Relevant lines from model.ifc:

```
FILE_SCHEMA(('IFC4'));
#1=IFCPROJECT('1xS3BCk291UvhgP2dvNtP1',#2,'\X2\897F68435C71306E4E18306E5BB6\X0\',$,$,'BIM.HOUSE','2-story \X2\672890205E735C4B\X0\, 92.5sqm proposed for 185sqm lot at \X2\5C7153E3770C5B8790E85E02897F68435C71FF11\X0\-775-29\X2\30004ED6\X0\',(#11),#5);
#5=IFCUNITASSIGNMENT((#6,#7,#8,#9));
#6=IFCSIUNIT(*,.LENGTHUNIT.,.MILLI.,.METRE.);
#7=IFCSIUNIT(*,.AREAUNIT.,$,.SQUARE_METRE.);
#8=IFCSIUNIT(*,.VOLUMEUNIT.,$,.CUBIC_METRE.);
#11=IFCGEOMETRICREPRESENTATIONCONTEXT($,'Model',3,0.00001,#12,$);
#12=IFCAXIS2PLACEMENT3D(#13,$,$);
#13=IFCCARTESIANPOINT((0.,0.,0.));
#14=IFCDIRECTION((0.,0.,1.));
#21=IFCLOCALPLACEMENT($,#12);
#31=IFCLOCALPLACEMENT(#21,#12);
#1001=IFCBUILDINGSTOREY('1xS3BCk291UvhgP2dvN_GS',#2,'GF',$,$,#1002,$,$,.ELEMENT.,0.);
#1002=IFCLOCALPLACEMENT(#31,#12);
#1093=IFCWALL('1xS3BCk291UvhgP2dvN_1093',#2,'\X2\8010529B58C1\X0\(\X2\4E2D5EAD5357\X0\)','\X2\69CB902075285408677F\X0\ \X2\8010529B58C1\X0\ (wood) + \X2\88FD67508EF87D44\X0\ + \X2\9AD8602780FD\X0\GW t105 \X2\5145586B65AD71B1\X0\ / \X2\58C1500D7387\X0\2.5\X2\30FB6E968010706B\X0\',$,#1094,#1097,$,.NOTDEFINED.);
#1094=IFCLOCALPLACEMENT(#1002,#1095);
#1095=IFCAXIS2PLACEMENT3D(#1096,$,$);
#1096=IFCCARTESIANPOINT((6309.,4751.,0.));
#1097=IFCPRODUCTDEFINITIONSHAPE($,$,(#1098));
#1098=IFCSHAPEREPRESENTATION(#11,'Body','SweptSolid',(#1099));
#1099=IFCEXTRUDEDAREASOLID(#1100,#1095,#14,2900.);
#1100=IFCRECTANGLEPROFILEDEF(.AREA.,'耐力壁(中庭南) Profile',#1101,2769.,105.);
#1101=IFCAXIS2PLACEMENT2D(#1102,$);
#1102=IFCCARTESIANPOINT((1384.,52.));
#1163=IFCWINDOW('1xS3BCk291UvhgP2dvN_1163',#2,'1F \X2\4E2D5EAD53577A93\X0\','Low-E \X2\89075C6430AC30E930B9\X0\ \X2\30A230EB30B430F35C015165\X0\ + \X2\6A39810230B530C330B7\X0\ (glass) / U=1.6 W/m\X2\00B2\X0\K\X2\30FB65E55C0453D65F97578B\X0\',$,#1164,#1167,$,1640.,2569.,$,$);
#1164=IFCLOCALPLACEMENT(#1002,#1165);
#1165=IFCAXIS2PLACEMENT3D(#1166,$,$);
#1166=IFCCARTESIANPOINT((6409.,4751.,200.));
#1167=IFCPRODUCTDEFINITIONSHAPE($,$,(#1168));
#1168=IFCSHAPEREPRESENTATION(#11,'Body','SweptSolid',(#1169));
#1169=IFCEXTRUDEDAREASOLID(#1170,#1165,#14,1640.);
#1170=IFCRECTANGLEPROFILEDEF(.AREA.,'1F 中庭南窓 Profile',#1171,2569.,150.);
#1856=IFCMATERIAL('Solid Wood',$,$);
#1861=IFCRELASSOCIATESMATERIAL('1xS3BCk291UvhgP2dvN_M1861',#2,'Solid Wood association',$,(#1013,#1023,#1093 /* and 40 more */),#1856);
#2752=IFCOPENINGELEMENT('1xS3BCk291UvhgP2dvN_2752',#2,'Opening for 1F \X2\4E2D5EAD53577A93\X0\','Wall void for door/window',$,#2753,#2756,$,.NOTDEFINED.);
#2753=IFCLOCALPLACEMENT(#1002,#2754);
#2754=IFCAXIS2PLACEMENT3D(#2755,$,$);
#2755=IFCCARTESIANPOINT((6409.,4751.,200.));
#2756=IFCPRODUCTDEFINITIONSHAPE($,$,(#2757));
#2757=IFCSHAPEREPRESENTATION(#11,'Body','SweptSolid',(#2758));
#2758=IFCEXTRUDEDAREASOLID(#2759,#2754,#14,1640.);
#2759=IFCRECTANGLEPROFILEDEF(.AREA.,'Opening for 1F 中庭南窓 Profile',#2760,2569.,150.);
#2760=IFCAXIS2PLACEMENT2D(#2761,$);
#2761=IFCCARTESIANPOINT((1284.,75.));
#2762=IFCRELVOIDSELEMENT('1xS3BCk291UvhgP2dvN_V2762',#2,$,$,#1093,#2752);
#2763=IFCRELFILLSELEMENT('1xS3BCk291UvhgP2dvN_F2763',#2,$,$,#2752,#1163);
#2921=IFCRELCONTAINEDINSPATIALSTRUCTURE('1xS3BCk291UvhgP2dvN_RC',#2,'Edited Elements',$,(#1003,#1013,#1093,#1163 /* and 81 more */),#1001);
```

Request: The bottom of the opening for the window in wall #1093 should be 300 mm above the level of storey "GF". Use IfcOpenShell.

```python
import numpy as np
import ifcopenshell
import ifcopenshell.api.geometry
import ifcopenshell.geom
import ifcopenshell.util.element
import ifcopenshell.util.placement
import ifcopenshell.util.shape
import ifcopenshell.util.unit

model = ifcopenshell.open("model.ifc")
unit_scale = ifcopenshell.util.unit.calculate_unit_scale(model)

window = model.by_id(1163)
opening = window.FillsVoids[0].RelatingOpeningElement
storey = ifcopenshell.util.element.get_container(window, ifc_class="IfcBuildingStorey")
level = ifcopenshell.util.placement.get_local_placement(storey.ObjectPlacement)[2, 3]

# The opening's origin need not be at the sill, so measure its lowest point.
shape = ifcopenshell.geom.create_shape(ifcopenshell.geom.settings(), opening)
bottom = ifcopenshell.util.shape.get_shape_bottom_elevation(shape, shape.geometry) / unit_scale
dz = level + 0.3 / unit_scale - bottom

shift = np.array([0.0, 0.0, dz])
# The window is not placed relative to its opening, so move both.
for product in (opening, window):
    matrix = ifcopenshell.util.placement.get_local_placement(product.ObjectPlacement)
    matrix[:3, 3] += shift
    ifcopenshell.api.geometry.edit_object_placement(model, product=product, matrix=matrix, is_si=False)

print(f"moved by {dz * unit_scale:+.3f} m")

model.write("model_v2.ifc")
```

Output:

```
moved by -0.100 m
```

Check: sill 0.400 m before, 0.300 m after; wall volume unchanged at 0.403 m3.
